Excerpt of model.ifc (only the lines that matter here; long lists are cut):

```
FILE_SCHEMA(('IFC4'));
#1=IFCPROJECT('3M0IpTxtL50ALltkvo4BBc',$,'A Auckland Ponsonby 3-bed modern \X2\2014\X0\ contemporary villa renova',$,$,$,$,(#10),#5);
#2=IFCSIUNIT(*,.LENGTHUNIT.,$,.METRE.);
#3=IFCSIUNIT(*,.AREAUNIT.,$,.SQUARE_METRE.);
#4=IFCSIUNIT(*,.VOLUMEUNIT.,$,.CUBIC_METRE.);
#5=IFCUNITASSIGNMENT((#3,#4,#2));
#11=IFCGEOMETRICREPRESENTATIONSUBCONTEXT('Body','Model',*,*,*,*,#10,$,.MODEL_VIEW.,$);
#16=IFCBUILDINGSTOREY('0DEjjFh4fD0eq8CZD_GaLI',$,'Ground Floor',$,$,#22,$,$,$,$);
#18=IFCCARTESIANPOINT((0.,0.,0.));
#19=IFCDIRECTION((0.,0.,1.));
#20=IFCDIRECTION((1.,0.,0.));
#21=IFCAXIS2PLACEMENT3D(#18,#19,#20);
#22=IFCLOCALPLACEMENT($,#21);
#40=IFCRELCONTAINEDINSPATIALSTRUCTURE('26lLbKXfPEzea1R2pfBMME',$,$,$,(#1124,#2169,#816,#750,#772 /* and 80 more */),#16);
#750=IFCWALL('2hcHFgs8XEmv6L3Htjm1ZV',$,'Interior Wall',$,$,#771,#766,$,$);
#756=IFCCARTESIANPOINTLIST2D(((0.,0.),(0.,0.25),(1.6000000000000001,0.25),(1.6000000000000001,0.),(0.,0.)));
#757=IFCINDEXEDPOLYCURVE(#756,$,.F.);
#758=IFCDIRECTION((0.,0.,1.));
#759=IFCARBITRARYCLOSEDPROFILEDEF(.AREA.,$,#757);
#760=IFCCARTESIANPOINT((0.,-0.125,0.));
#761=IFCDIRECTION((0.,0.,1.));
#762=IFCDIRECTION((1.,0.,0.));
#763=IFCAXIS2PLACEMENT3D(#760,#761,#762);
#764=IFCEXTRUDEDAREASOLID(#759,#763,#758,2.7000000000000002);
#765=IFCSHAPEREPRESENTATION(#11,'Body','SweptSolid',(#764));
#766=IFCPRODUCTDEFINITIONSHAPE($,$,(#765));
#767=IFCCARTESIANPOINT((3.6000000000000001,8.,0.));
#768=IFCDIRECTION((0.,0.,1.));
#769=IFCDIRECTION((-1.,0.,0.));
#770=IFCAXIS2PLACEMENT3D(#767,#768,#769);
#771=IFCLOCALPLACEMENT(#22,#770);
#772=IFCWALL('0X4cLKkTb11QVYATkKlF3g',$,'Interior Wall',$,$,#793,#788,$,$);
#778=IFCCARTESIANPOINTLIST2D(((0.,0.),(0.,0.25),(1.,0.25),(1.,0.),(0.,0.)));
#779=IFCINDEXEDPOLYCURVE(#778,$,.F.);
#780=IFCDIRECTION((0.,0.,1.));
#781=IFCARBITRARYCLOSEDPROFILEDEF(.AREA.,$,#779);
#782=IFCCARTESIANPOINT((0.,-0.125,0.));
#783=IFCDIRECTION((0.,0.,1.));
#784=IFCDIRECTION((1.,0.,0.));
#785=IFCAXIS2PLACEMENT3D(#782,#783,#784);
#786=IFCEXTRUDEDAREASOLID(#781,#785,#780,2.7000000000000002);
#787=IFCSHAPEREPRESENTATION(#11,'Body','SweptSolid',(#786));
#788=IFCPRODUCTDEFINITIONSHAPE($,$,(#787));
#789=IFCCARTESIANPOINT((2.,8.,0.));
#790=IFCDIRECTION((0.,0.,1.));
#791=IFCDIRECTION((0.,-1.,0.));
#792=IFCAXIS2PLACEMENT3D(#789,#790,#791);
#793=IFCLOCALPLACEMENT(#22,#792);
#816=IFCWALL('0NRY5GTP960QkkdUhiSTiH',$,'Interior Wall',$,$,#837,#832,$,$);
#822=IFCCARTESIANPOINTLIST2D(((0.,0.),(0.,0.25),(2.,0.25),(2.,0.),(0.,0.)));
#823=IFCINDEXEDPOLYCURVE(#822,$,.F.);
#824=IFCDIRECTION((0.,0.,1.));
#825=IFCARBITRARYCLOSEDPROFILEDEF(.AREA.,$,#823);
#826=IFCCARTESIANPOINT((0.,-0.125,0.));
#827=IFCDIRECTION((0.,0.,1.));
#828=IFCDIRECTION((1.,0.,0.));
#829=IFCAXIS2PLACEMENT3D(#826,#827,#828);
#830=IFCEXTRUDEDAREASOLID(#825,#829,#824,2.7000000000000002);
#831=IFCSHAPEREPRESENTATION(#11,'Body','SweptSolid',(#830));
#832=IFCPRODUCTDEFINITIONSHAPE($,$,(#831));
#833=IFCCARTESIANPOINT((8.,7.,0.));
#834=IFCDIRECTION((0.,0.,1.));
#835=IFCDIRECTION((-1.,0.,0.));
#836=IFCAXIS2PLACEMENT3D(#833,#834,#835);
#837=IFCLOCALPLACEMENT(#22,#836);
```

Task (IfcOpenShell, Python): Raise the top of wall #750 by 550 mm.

```python
import ifcopenshell
import ifcopenshell.geom
import ifcopenshell.util.representation
import ifcopenshell.util.shape
import ifcopenshell.util.unit

model = ifcopenshell.open("model.ifc")
unit_scale = ifcopenshell.util.unit.calculate_unit_scale(model)
settings = ifcopenshell.geom.settings()


def volume(element):
    """Net volume in cubic metres, openings subtracted."""
    shape = ifcopenshell.geom.create_shape(settings, element)
    return ifcopenshell.util.shape.get_volume(shape.geometry)


wall = model.by_guid("2hcHFgs8XEmv6L3Htjm1ZV")
before = volume(wall)

body = ifcopenshell.util.representation.get_representation(wall, "Model", "Body")
solid = body.Items[0]
old_height = solid.Depth
solid.Depth += 0.55 / unit_scale
after = volume(wall)

print(f"height {old_height:g} -> {solid.Depth:g}, volume {before:.3f} -> {after:.3f} m3")

model.write("model_rev.ifc")
```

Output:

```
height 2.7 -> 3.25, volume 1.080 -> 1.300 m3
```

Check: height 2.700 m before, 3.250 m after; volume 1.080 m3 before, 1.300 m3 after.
